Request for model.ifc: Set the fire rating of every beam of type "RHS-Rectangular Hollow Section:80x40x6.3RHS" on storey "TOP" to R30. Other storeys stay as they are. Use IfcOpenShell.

First a look at what the model holds.

```python
import ifcopenshell
import ifcopenshell.util.element

model = ifcopenshell.open("model.ifc")
print(model.schema)
storey = next(s for s in model.by_type("IfcBuildingStorey") if s.Name == "TOP")
beams = [e for e in ifcopenshell.util.element.get_decomposition(storey) if e.is_a("IfcBeam")]
seen = {}
for e in beams:
    element_type = ifcopenshell.util.element.get_type(e)
    key = (element_type.Name if element_type != e and element_type else None, ifcopenshell.util.element.get_pset(e, "Pset_BeamCommon", "FireRating"))
    seen[key] = seen.get(key, 0) + 1
for (name, value), count in sorted(seen.items(), key=str):
    print(count, "x", name, "|", value)
```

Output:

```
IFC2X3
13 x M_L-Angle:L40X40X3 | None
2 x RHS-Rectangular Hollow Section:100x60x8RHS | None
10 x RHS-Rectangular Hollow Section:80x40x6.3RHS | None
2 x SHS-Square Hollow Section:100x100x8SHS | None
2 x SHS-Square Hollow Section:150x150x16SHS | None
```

```python
import ifcopenshell
import ifcopenshell.api.pset
import ifcopenshell.util.element

model = ifcopenshell.open("model.ifc")

storey = next(s for s in model.by_type("IfcBuildingStorey") if s.Name == "TOP")
beams = [e for e in ifcopenshell.util.element.get_decomposition(storey) if e.is_a("IfcBeam")]

count = 0
for e in beams:
    element_type = ifcopenshell.util.element.get_type(e)
    if element_type in (None, e) or element_type.Name != "RHS-Rectangular Hollow Section:80x40x6.3RHS":
        continue
    # add_pset returns the element's existing set when there is one.
    pset = ifcopenshell.api.pset.add_pset(model, product=e, name="Pset_BeamCommon")
    ifcopenshell.api.pset.edit_pset(model, pset=pset, properties={"FireRating": "R30"})
    count += 1

print(count, "beams updated")

model.write("model_updated.ifc")
```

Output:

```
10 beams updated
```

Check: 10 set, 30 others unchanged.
